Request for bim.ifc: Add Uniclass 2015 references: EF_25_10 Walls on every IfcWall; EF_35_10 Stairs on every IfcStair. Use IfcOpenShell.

First a look at what the model holds.

```python
import ifcopenshell

model = ifcopenshell.open("bim.ifc")
print(model.schema)
print("classifications:", [c.Name for c in model.by_type("IfcClassification")])
for ifc_class in ("IfcDoor", "IfcRoof", "IfcStair", "IfcWall", "IfcWindow"):
    print(ifc_class, len(model.by_type(ifc_class)))
```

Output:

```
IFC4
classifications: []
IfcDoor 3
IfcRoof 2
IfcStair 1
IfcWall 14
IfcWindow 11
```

```python
import ifcopenshell
import ifcopenshell.api.classification

model = ifcopenshell.open("bim.ifc")

system = ifcopenshell.api.classification.add_classification(model, classification="Uniclass 2015")

codes = {
    "IfcWall": ("EF_25_10", "Walls"),
    "IfcStair": ("EF_35_10", "Stairs"),
}
for ifc_class, (code, name) in codes.items():
    products = model.by_type(ifc_class)
    ifcopenshell.api.classification.add_reference(
        model, products=products, classification=system, identification=code, name=name
    )
    print(code, len(products))

model.write("bim_updated.ifc")
```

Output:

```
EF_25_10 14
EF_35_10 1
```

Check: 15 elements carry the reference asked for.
